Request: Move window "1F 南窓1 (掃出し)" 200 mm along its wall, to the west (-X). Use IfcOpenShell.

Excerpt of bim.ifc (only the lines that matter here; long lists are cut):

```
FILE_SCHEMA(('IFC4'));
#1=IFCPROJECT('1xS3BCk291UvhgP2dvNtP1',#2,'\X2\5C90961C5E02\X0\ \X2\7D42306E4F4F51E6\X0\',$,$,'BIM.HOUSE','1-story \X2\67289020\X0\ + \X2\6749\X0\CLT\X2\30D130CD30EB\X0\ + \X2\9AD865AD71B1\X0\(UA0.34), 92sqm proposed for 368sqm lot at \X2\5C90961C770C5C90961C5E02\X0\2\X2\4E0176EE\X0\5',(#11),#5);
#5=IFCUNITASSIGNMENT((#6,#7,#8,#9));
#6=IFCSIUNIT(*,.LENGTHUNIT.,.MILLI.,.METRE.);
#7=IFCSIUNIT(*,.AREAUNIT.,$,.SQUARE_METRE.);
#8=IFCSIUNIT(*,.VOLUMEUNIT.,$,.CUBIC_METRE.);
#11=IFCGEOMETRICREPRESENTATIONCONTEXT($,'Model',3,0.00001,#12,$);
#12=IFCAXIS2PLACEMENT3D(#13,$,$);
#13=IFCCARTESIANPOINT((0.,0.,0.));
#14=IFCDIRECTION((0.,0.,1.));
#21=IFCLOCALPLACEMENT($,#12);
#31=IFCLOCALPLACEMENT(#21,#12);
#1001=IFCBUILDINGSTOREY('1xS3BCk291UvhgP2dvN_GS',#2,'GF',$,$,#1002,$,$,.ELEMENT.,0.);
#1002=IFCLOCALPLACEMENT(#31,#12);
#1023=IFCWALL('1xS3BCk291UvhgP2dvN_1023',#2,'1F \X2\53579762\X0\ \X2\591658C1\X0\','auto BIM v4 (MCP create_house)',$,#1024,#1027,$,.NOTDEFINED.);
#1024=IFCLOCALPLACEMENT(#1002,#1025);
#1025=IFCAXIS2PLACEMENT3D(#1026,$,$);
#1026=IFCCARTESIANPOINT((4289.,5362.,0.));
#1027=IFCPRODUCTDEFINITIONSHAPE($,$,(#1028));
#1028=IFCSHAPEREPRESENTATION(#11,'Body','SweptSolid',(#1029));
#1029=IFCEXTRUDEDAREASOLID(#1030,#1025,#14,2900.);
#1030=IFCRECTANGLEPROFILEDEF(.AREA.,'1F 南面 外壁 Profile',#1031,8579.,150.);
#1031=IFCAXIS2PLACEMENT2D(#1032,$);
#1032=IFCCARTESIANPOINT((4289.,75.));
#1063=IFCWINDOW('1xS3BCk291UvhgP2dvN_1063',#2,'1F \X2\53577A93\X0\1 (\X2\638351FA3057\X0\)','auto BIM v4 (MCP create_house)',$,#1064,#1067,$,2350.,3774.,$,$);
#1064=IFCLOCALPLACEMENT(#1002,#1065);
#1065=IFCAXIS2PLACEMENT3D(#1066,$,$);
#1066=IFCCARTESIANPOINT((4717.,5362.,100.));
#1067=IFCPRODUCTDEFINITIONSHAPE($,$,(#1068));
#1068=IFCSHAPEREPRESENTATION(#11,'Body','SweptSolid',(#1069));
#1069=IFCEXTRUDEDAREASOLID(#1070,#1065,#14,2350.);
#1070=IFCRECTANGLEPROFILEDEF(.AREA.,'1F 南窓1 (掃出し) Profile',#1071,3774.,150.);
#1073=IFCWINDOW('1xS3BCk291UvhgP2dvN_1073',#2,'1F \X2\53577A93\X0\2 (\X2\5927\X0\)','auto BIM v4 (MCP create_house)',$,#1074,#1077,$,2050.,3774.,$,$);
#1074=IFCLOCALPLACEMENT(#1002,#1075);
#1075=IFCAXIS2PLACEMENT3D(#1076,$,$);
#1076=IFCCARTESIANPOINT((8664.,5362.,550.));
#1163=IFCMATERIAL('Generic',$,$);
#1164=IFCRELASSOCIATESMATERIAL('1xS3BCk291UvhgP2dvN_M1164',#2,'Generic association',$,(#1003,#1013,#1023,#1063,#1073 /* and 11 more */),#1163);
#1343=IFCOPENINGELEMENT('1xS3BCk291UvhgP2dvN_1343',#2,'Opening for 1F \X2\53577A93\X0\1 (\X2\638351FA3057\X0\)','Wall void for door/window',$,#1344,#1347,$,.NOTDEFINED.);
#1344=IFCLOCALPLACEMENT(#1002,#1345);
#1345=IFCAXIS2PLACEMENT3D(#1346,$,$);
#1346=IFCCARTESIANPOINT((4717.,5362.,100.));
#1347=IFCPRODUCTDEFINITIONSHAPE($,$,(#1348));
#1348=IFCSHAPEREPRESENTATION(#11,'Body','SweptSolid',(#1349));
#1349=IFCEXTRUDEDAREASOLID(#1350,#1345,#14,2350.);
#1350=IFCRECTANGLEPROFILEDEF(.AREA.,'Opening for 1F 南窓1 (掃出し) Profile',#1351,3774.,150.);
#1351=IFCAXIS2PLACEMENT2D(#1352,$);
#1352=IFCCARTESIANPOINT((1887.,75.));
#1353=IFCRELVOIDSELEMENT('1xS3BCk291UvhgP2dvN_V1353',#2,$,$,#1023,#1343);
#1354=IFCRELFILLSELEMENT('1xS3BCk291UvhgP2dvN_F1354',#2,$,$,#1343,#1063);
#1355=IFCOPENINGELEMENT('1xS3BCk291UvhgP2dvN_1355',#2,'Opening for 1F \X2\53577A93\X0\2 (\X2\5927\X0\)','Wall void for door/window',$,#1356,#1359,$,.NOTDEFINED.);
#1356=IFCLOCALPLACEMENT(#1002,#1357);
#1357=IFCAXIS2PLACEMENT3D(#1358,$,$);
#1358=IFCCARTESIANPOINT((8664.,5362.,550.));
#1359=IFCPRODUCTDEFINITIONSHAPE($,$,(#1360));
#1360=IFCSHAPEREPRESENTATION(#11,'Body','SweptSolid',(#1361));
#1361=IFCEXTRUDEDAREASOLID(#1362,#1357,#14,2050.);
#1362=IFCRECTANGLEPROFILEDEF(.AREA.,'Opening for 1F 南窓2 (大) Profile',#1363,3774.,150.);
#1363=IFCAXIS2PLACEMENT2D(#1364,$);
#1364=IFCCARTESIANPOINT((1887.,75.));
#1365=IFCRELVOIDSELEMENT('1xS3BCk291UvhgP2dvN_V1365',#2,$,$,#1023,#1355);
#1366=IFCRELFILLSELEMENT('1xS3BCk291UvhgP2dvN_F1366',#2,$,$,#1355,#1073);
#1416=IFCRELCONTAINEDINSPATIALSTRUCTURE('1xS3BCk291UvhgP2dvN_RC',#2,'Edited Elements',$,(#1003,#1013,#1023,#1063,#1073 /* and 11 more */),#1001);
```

```python
import ifcopenshell
import ifcopenshell.api.geometry
import ifcopenshell.util.placement
import ifcopenshell.util.unit

model = ifcopenshell.open("bim.ifc")
unit_scale = ifcopenshell.util.unit.calculate_unit_scale(model)

window = model.by_id(1063)
opening = window.FillsVoids[0].RelatingOpeningElement
wall = opening.VoidsElements[0].RelatingBuildingElement

wall_matrix = ifcopenshell.util.placement.get_local_placement(wall.ObjectPlacement)
shift = wall_matrix[:3, 0] * -0.2 / unit_scale
before = ifcopenshell.util.placement.get_local_placement(window.ObjectPlacement)[:3, 3].copy()

# The window is not placed relative to its opening, so move both.
for product in (opening, window):
    matrix = ifcopenshell.util.placement.get_local_placement(product.ObjectPlacement)
    matrix[:3, 3] += shift
    ifcopenshell.api.geometry.edit_object_placement(model, product=product, matrix=matrix, is_si=False)

after = ifcopenshell.util.placement.get_local_placement(window.ObjectPlacement)[:3, 3]
print("window moved by", (after - before).round(3) + 0.0)

model.write("bim-out.ifc")
```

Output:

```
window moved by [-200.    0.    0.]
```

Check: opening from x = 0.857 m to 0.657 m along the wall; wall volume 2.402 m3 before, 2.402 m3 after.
